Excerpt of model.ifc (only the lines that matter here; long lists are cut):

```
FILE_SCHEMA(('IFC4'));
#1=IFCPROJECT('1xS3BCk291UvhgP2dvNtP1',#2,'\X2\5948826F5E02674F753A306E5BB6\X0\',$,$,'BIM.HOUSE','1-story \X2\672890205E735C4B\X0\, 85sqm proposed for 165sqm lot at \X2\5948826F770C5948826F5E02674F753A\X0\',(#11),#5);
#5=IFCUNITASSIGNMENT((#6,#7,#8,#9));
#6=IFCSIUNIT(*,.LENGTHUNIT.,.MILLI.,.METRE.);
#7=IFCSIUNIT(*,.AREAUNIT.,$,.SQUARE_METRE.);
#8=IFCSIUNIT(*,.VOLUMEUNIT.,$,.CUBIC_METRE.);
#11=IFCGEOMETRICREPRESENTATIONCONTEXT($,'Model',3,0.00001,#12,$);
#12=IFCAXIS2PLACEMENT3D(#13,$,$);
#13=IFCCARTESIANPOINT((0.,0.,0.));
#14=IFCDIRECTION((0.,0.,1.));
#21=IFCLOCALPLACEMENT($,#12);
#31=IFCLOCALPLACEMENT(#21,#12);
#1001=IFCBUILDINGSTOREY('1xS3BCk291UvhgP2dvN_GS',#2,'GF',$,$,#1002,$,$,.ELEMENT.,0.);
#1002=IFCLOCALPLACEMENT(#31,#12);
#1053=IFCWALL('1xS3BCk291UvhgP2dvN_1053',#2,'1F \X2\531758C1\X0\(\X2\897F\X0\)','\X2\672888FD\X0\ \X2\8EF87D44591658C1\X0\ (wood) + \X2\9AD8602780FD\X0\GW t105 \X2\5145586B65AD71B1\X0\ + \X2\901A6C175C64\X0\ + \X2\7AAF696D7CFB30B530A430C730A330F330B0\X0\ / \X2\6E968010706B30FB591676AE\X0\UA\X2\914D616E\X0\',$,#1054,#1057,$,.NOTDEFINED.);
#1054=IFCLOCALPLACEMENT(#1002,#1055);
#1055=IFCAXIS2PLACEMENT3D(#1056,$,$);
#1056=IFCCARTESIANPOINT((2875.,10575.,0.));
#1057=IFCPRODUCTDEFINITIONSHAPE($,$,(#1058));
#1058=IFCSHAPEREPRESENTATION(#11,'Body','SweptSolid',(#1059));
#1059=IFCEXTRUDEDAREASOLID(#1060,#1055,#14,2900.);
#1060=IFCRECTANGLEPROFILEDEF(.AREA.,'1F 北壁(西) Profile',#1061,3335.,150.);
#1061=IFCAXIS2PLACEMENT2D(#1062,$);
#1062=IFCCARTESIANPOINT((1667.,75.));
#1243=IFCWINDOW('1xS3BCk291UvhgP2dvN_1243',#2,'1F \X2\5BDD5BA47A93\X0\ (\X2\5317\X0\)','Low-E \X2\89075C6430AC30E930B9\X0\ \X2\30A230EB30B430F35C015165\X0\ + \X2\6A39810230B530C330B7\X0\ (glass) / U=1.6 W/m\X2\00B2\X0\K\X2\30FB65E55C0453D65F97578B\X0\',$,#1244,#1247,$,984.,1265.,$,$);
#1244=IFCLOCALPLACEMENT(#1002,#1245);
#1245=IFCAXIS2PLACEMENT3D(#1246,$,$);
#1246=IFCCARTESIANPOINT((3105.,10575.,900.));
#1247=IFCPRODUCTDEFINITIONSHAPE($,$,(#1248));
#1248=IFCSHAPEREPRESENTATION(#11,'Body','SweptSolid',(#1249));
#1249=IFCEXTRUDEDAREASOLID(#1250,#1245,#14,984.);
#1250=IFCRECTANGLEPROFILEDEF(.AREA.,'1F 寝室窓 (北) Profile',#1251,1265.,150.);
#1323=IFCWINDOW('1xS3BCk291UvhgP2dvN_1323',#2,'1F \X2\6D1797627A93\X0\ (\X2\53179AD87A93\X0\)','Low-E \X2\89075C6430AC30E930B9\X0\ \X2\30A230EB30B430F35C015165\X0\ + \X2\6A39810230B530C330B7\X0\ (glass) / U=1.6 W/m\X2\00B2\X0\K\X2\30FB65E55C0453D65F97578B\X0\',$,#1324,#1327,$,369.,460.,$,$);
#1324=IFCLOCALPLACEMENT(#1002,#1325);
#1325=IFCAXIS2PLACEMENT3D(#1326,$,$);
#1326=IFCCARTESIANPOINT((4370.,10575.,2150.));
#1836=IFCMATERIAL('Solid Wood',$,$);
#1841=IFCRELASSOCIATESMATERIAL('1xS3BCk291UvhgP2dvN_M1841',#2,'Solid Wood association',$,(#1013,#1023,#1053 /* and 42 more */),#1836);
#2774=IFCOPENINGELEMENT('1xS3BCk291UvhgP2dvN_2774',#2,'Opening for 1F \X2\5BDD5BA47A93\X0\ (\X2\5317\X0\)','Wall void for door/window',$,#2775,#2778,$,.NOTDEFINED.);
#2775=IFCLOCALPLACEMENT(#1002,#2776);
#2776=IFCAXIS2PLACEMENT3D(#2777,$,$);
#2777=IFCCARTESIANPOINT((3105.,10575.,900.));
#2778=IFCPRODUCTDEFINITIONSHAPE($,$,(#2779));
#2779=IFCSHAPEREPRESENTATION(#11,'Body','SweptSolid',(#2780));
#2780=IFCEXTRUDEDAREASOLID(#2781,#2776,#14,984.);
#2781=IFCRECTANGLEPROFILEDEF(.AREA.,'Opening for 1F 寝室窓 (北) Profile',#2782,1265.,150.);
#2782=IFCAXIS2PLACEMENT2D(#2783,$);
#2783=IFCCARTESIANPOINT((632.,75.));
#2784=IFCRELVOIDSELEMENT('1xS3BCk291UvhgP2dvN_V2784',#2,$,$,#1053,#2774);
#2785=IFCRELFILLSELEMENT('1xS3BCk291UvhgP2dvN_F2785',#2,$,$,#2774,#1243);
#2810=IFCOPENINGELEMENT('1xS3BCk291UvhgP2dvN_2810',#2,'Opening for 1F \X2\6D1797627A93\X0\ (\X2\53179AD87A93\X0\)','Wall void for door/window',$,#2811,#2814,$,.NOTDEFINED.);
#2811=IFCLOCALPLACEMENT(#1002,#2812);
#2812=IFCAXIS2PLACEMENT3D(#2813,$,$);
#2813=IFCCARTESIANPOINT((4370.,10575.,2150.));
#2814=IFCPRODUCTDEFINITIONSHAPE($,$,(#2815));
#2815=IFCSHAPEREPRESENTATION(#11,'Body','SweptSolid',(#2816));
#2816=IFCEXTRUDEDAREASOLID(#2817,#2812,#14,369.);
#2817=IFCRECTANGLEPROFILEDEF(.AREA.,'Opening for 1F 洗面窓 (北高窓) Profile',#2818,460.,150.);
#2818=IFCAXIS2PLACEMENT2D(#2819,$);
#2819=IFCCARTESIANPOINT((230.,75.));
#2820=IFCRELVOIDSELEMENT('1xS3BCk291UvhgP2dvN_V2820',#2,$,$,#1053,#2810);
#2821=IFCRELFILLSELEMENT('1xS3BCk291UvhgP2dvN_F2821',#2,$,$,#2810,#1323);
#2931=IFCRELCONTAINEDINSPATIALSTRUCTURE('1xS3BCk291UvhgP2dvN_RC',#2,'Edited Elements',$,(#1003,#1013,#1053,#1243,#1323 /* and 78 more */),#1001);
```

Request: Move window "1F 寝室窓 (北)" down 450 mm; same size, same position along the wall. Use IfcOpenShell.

```python
import numpy as np
import ifcopenshell
import ifcopenshell.api.geometry
import ifcopenshell.util.placement
import ifcopenshell.util.unit

model = ifcopenshell.open("model.ifc")
unit_scale = ifcopenshell.util.unit.calculate_unit_scale(model)

window = model.by_guid("1xS3BCk291UvhgP2dvN_1243")
opening = window.FillsVoids[0].RelatingOpeningElement
dz = -450.0

shift = np.array([0.0, 0.0, dz])
# The window is not placed relative to its opening, so move both.
for product in (opening, window):
    matrix = ifcopenshell.util.placement.get_local_placement(product.ObjectPlacement)
    matrix[:3, 3] += shift
    ifcopenshell.api.geometry.edit_object_placement(model, product=product, matrix=matrix, is_si=False)

print(f"moved by {dz * unit_scale:+.3f} m")

model.write("model_edited.ifc")
```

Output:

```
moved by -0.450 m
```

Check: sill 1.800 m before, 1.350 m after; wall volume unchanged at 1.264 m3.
